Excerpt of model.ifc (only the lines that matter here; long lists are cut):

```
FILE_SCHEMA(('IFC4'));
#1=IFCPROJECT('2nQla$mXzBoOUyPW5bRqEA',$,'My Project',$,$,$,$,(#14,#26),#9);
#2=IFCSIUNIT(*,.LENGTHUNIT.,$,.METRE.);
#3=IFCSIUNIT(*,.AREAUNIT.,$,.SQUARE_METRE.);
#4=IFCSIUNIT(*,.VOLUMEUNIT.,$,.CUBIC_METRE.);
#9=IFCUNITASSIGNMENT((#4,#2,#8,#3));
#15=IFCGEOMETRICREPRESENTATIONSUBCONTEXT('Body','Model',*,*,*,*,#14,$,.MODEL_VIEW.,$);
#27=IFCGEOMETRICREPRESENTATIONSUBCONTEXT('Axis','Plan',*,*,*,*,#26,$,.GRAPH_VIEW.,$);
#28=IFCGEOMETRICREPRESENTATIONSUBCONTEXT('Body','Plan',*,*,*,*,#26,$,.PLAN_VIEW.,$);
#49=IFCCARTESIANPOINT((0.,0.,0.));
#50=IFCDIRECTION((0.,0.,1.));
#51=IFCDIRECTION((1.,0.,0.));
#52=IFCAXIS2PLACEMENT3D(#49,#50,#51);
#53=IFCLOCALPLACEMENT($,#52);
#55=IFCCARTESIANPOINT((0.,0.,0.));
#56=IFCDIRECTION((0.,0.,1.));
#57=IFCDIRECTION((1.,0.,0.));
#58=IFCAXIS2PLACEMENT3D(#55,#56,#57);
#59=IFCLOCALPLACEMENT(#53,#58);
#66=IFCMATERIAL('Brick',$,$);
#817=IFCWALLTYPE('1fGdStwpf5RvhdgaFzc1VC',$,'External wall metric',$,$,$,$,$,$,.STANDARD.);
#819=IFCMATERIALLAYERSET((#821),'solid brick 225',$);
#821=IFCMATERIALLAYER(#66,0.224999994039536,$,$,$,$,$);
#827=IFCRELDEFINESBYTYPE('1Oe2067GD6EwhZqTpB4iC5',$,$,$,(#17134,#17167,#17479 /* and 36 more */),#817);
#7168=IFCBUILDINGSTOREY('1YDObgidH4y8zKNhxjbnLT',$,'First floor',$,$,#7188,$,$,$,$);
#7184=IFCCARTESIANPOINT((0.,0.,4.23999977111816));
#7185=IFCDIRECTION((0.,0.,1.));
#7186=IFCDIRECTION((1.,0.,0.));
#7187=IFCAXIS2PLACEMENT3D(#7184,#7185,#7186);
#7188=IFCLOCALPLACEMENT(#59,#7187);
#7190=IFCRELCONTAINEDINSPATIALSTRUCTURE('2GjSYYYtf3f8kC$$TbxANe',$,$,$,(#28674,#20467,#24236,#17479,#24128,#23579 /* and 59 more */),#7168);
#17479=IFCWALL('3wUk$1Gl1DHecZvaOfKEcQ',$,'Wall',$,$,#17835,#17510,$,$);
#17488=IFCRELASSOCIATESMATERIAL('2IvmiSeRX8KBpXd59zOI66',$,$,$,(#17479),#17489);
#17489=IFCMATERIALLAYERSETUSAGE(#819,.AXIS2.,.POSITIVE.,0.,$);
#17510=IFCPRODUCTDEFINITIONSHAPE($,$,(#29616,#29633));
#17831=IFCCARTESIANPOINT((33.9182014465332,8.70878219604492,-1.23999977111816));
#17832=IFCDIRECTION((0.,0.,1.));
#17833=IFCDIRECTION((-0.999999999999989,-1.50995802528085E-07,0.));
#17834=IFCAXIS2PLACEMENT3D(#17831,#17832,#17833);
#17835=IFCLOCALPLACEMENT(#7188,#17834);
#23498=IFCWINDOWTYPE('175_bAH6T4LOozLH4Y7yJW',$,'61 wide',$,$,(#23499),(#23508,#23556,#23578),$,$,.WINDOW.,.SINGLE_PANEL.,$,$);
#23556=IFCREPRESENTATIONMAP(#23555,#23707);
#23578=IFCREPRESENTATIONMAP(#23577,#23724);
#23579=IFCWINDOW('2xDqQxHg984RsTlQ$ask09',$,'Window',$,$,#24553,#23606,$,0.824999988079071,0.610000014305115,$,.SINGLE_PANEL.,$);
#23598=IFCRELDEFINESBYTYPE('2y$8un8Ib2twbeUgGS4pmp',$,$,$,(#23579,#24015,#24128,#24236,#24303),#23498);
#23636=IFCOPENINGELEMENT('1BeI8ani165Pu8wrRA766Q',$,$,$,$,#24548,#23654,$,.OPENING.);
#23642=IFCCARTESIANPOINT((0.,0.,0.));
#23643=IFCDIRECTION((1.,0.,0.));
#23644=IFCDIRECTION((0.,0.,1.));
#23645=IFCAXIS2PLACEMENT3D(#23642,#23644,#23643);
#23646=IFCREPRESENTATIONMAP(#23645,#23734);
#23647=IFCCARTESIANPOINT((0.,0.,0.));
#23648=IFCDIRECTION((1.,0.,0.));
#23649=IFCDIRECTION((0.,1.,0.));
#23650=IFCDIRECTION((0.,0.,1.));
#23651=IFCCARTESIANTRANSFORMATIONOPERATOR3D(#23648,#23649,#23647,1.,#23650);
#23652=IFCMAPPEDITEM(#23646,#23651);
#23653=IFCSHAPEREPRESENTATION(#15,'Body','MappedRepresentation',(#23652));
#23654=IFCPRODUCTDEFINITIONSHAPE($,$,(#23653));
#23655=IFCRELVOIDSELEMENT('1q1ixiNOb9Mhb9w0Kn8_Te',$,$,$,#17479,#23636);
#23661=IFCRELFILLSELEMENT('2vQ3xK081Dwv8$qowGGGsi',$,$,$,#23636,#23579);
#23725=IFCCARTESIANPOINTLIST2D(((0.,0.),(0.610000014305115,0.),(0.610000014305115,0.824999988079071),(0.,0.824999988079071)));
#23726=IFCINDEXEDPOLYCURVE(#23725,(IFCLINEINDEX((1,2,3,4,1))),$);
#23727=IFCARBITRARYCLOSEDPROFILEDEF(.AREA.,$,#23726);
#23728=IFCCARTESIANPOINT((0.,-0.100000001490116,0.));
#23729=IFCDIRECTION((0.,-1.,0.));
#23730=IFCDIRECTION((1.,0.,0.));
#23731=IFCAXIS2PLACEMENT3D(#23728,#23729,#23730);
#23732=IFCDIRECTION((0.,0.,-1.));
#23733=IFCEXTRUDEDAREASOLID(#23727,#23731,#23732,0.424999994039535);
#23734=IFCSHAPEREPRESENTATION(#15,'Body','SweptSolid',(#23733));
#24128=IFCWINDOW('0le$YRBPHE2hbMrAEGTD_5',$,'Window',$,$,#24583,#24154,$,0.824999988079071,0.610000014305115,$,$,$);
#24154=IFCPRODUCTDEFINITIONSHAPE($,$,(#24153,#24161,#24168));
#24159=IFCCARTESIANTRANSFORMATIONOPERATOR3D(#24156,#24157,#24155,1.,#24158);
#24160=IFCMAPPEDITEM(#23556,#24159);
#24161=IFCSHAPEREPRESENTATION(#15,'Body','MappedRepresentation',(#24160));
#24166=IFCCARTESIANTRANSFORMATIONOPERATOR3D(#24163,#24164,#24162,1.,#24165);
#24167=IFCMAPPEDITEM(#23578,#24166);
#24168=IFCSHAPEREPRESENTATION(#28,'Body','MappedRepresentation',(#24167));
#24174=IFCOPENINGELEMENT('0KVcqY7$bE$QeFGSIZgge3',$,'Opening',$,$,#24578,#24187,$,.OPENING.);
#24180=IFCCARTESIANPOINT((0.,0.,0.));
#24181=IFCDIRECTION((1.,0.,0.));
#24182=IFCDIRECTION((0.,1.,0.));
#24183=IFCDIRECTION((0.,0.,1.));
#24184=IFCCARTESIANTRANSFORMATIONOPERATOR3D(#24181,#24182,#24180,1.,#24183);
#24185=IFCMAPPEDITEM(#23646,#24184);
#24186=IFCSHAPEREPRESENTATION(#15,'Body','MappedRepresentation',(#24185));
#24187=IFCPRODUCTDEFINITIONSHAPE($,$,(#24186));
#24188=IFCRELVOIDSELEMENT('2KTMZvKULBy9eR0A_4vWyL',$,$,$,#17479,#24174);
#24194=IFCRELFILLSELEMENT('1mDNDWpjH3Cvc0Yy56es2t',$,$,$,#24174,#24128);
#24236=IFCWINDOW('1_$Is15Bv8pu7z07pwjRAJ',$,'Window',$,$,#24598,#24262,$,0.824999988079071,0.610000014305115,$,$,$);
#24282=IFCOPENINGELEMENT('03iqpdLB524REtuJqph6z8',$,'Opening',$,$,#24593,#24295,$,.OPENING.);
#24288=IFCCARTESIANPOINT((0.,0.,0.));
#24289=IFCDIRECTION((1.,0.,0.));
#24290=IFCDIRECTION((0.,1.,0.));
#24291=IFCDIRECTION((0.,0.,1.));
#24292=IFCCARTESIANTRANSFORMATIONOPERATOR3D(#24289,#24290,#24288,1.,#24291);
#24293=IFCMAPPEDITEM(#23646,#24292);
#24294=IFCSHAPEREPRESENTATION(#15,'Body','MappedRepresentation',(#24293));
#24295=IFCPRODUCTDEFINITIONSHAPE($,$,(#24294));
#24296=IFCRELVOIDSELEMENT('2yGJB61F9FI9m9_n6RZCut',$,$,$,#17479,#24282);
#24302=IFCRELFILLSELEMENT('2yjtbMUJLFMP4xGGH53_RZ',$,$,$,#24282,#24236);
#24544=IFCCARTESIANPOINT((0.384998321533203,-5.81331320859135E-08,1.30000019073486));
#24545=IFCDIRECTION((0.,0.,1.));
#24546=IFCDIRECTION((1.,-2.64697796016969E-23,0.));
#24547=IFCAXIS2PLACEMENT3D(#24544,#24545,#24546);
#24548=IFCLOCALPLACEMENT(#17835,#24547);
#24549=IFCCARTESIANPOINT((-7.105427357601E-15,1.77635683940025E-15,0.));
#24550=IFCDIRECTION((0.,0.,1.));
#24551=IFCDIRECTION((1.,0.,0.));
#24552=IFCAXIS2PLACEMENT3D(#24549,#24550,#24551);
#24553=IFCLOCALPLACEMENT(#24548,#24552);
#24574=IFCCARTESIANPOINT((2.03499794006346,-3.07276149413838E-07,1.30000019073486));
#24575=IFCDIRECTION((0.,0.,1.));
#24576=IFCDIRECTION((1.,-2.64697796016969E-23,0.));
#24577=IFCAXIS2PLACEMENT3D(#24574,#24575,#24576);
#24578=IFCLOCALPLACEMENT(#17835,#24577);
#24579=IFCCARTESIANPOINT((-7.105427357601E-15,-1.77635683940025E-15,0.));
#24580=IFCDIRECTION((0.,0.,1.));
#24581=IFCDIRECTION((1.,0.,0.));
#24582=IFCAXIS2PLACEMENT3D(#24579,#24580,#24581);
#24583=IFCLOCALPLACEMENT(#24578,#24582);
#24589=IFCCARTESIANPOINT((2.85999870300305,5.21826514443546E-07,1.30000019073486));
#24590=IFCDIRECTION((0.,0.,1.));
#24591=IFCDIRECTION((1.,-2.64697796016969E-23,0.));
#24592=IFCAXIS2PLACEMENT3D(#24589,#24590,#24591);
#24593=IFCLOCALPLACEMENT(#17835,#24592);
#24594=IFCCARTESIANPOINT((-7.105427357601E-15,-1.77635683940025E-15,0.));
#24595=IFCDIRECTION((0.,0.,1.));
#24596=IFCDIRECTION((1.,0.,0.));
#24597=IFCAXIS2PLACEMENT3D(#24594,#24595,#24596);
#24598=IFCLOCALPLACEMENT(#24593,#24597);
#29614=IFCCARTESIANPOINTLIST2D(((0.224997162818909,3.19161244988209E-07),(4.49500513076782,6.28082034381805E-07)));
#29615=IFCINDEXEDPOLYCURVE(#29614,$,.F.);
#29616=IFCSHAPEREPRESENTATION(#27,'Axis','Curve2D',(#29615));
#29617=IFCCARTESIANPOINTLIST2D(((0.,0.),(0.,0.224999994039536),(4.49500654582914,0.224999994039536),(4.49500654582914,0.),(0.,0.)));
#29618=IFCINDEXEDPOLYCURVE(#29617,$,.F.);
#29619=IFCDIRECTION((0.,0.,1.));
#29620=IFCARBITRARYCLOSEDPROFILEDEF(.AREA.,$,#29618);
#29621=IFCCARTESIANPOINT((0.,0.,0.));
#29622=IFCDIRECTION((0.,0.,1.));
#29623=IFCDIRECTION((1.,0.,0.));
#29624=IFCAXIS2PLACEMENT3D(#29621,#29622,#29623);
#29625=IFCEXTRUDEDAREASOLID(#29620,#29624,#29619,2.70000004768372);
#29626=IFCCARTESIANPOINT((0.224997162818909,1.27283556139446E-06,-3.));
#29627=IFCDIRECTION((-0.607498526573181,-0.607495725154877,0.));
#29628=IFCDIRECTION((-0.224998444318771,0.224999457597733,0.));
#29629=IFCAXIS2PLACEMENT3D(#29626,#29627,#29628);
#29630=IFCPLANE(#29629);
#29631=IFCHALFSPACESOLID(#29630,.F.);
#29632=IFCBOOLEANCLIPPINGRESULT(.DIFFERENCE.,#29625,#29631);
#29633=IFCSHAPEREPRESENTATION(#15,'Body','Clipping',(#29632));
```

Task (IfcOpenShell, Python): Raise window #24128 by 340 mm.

```python
import numpy as np
import ifcopenshell
import ifcopenshell.api.geometry
import ifcopenshell.util.placement
import ifcopenshell.util.unit

model = ifcopenshell.open("model.ifc")
unit_scale = ifcopenshell.util.unit.calculate_unit_scale(model)

window = model.by_guid("0le$YRBPHE2hbMrAEGTD_5")
opening = window.FillsVoids[0].RelatingOpeningElement
dz = 0.34 / unit_scale

shift = np.array([0.0, 0.0, dz])
# The window is placed relative to its opening, so it follows when the opening moves.
matrix = ifcopenshell.util.placement.get_local_placement(opening.ObjectPlacement)
matrix[:3, 3] += shift
ifcopenshell.api.geometry.edit_object_placement(
    model, product=opening, matrix=matrix, is_si=False, should_transform_children=True
)

print(f"moved by {dz * unit_scale:+.3f} m")

model.write("model-out.ifc")
```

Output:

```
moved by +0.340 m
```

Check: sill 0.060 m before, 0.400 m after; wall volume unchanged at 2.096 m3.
